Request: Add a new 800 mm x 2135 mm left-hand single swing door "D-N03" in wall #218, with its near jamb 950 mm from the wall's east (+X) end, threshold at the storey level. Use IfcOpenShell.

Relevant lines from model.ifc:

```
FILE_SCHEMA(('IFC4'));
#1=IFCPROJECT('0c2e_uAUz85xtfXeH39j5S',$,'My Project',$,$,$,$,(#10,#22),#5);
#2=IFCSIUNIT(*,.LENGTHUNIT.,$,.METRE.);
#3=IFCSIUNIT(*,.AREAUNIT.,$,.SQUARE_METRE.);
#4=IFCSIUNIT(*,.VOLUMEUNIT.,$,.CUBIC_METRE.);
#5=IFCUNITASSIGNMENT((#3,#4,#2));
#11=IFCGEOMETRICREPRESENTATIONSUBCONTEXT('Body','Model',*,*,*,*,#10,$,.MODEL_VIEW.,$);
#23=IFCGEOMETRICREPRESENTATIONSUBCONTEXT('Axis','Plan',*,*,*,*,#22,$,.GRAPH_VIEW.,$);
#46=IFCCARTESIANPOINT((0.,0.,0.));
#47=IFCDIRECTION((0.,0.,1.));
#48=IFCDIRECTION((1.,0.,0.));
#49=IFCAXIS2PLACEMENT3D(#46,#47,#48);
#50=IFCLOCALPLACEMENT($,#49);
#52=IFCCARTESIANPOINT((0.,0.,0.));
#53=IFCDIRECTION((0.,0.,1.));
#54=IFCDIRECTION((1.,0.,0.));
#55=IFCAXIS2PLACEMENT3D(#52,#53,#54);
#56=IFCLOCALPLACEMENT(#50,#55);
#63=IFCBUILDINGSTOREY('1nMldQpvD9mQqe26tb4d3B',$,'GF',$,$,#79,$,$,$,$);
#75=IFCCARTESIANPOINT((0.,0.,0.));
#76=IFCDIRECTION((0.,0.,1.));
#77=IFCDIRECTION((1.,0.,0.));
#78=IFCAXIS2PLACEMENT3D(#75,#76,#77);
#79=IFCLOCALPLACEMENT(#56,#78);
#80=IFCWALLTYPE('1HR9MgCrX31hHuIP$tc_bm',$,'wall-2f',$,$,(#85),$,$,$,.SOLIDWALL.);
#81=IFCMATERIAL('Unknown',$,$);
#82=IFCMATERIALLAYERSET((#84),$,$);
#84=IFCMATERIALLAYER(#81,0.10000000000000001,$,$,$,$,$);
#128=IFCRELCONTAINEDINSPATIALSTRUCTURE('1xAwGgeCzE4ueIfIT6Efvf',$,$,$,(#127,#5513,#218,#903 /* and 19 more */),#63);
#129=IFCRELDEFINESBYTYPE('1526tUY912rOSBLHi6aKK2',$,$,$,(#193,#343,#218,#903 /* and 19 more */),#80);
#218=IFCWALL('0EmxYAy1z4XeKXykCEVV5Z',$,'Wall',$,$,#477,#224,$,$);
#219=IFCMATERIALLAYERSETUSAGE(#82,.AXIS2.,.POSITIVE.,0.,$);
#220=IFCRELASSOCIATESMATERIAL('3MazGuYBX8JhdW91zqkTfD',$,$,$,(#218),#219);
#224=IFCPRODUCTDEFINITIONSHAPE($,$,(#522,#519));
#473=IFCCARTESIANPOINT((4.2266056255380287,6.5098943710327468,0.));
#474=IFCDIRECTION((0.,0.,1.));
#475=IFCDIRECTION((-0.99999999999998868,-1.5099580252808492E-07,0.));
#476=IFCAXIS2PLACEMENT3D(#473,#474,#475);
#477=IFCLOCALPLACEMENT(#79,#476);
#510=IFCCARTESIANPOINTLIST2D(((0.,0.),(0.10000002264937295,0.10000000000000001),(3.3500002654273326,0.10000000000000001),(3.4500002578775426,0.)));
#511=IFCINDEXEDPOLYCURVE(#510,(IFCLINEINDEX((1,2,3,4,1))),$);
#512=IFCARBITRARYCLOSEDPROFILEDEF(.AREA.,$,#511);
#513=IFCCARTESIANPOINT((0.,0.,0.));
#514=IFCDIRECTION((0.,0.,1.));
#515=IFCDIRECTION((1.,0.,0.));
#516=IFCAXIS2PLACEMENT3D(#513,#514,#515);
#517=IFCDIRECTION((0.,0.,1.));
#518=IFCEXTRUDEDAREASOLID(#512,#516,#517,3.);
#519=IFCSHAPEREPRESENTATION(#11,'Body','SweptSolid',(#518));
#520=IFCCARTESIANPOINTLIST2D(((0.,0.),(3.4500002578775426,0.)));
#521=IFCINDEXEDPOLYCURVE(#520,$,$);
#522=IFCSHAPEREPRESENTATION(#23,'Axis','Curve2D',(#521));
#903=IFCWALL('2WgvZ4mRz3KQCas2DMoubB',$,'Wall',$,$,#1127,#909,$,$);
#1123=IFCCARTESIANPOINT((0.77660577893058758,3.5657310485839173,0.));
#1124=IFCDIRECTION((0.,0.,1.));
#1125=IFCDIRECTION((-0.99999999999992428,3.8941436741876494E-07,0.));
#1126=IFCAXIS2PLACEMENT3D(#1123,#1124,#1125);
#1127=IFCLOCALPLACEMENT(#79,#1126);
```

```python
import numpy as np
import ifcopenshell
import ifcopenshell.api.feature
import ifcopenshell.api.geometry
import ifcopenshell.api.root
import ifcopenshell.api.spatial
import ifcopenshell.geom
import ifcopenshell.util.element
import ifcopenshell.util.placement
import ifcopenshell.util.representation
import ifcopenshell.util.shape
import ifcopenshell.util.unit

model = ifcopenshell.open("model.ifc")
unit_scale = ifcopenshell.util.unit.calculate_unit_scale(model)
settings = ifcopenshell.geom.settings()


def volume(element):
    """Net volume in cubic metres, openings subtracted."""
    shape = ifcopenshell.geom.create_shape(settings, element)
    return ifcopenshell.util.shape.get_volume(shape.geometry)


wall = model.by_guid("0EmxYAy1z4XeKXykCEVV5Z")
storey = ifcopenshell.util.element.get_container(wall, ifc_class="IfcBuildingStorey")
context = ifcopenshell.util.representation.get_context(model, "Model", "Body", "MODEL_VIEW")
before = volume(wall)

width, height, from_end, sill = 0.8, 2.135, 0.95, 0.0  # metres

# The wall runs along its own X axis, and the end named is its -X end.
wall_shape = ifcopenshell.geom.create_shape(settings, wall)
x, y, z = ifcopenshell.util.shape.get_vertices(wall_shape.geometry).T
start = x.min() + from_end
face, thickness = float(y.min()), float(y.max() - y.min())
wall_matrix = ifcopenshell.util.placement.get_local_placement(wall.ObjectPlacement)
level = ifcopenshell.util.placement.get_local_placement(storey.ObjectPlacement)[2, 3]


def in_wall(x, y):
    """Placement at x, y metres in the wall's axes, at sill height."""
    matrix = wall_matrix.copy()
    matrix[:, 3] = wall_matrix @ np.array([x / unit_scale, y / unit_scale, 0.0, 1.0])
    matrix[2, 3] = level + sill / unit_scale
    return matrix


# Opening: a box that overshoots both wall faces by 50 mm.
opening = ifcopenshell.api.root.create_entity(model, ifc_class="IfcOpeningElement", predefined_type="OPENING")
box = ifcopenshell.api.geometry.add_wall_representation(
    model, context=context, length=width, height=height, thickness=thickness + 0.1
)
ifcopenshell.api.geometry.assign_representation(model, product=opening, representation=box)
ifcopenshell.api.geometry.edit_object_placement(model, product=opening, matrix=in_wall(start, face - 0.05), is_si=False)
ifcopenshell.api.feature.add_feature(model, feature=opening, element=wall)

door = ifcopenshell.api.root.create_entity(model, ifc_class="IfcDoor", name="D-N03", predefined_type="DOOR")
door.OverallWidth, door.OverallHeight = width / unit_scale, height / unit_scale
door.OperationType = "SINGLE_SWING_LEFT"
body = ifcopenshell.api.geometry.add_door_representation(
    model,
    context=context,
    overall_width=door.OverallWidth,
    overall_height=door.OverallHeight,
    operation_type="SINGLE_SWING_LEFT",
    lining_properties={"LiningDepth": thickness / unit_scale, "ThresholdDepth": thickness / unit_scale},
)
ifcopenshell.api.geometry.assign_representation(model, product=door, representation=body)
ifcopenshell.api.spatial.assign_container(model, products=[door], relating_structure=storey)
ifcopenshell.api.feature.add_filling(model, opening=opening, element=door)

# The lining spans the wall, so the door starts at the wall face.
ifcopenshell.api.geometry.edit_object_placement(model, product=door, matrix=in_wall(start, face), is_si=False)

after = volume(wall)

print(f"wall volume {before:.3f} -> {after:.3f} m3")

model.write("model-out.ifc")
```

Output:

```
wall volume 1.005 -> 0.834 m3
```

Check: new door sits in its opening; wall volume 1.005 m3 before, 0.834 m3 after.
